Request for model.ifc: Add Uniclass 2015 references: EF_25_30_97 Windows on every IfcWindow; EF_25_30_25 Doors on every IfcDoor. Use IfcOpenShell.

First a look at what the model holds.

```python
import ifcopenshell

model = ifcopenshell.open("model.ifc")
print(model.schema)
print("classifications:", [c.Name for c in model.by_type("IfcClassification")])
for ifc_class in ("IfcDoor", "IfcRoof", "IfcStair", "IfcWall", "IfcWindow"):
    print(ifc_class, len(model.by_type(ifc_class)))
```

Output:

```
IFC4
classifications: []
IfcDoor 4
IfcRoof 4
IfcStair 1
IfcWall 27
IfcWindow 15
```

```python
import ifcopenshell
import ifcopenshell.api.classification

model = ifcopenshell.open("model.ifc")

system = ifcopenshell.api.classification.add_classification(model, classification="Uniclass 2015")

codes = {
    "IfcWindow": ("EF_25_30_97", "Windows"),
    "IfcDoor": ("EF_25_30_25", "Doors"),
}
for ifc_class, (code, name) in codes.items():
    products = model.by_type(ifc_class)
    ifcopenshell.api.classification.add_reference(
        model, products=products, classification=system, identification=code, name=name
    )
    print(code, len(products))

model.write("model_v2.ifc")
```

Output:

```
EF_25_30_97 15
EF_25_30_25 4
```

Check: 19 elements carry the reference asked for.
